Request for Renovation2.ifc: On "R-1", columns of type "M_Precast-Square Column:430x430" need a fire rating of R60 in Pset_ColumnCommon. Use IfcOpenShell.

First a look at what the model holds.

```python
import ifcopenshell
import ifcopenshell.util.element

model = ifcopenshell.open("Renovation2.ifc")
print(model.schema)
storey = next(s for s in model.by_type("IfcBuildingStorey") if s.Name == "R-1")
columns = [e for e in ifcopenshell.util.element.get_decomposition(storey) if e.is_a("IfcColumn")]
seen = {}
for e in columns:
    element_type = ifcopenshell.util.element.get_type(e)
    key = (element_type.Name if element_type != e and element_type else None, ifcopenshell.util.element.get_pset(e, "Pset_ColumnCommon", "FireRating"))
    seen[key] = seen.get(key, 0) + 1
for (name, value), count in sorted(seen.items(), key=str):
    print(count, "x", name, "|", value)
```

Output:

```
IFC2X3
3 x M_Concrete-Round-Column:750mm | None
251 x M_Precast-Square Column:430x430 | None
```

```python
import ifcopenshell
import ifcopenshell.api.pset
import ifcopenshell.util.element

model = ifcopenshell.open("Renovation2.ifc")

storey = next(s for s in model.by_type("IfcBuildingStorey") if s.Name == "R-1")
columns = [e for e in ifcopenshell.util.element.get_decomposition(storey) if e.is_a("IfcColumn")]

count = 0
for e in columns:
    element_type = ifcopenshell.util.element.get_type(e)
    if element_type in (None, e) or element_type.Name != "M_Precast-Square Column:430x430":
        continue
    # add_pset returns the element's existing set when there is one.
    pset = ifcopenshell.api.pset.add_pset(model, product=e, name="Pset_ColumnCommon")
    ifcopenshell.api.pset.edit_pset(model, pset=pset, properties={"FireRating": "R60"})
    count += 1

print(count, "columns updated")

model.write("Renovation2-out.ifc")
```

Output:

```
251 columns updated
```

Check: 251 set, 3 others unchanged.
